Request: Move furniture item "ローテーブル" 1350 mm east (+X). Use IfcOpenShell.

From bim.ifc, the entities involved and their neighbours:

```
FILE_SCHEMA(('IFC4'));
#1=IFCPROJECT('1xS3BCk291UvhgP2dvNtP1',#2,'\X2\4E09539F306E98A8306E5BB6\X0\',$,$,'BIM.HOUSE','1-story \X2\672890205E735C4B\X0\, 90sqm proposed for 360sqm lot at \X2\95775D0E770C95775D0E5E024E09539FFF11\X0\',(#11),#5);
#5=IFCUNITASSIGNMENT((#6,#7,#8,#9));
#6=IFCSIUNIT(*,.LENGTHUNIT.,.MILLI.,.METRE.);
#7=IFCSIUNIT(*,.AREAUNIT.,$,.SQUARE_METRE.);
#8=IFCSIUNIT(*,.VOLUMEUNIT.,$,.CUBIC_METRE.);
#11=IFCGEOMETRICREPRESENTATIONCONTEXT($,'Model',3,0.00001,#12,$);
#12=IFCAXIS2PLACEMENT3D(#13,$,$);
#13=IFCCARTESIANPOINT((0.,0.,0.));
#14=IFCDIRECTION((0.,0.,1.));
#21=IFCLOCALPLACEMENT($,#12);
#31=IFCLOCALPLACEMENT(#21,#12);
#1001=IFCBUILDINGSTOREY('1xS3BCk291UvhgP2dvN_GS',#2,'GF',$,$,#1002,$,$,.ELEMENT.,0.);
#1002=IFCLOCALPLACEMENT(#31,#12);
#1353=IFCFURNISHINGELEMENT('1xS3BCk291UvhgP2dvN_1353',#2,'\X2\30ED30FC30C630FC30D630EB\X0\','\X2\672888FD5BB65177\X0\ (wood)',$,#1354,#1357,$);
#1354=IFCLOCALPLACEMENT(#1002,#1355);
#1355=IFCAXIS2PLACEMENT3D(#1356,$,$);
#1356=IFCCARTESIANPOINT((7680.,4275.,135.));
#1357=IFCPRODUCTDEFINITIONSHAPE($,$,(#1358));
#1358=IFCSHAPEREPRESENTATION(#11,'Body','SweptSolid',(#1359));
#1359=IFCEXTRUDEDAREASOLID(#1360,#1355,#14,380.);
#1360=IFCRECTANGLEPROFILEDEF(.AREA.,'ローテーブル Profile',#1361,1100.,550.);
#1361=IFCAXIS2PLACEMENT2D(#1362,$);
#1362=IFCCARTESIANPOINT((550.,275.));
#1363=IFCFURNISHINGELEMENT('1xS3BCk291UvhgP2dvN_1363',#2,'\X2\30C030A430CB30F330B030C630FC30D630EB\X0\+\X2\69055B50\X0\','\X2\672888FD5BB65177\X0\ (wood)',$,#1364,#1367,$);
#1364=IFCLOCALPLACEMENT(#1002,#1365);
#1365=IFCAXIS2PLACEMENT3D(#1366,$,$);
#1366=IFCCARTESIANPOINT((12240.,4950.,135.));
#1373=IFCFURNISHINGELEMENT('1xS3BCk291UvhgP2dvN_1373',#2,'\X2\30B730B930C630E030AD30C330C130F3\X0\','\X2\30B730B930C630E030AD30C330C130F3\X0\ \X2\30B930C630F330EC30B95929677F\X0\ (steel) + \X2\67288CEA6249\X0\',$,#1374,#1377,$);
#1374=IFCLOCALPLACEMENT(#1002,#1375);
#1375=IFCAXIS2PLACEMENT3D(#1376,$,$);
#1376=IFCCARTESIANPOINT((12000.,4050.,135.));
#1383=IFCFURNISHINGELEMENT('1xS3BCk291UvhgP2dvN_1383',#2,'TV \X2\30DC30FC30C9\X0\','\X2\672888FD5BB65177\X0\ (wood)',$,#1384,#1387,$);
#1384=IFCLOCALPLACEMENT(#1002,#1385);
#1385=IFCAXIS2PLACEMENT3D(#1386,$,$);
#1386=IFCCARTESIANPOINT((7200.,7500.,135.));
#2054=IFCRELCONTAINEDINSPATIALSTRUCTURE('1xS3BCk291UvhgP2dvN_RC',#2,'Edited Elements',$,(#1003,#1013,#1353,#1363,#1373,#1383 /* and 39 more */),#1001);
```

```python
import ifcopenshell
import ifcopenshell.api.geometry
import ifcopenshell.util.placement

model = ifcopenshell.open("bim.ifc")

item = model.by_guid("1xS3BCk291UvhgP2dvN_1353")
matrix = ifcopenshell.util.placement.get_local_placement(item.ObjectPlacement)
matrix[0, 3] += 1350.0
ifcopenshell.api.geometry.edit_object_placement(model, product=item, matrix=matrix, is_si=False)

print(ifcopenshell.util.placement.get_local_placement(item.ObjectPlacement).round(3) + 0.0)

model.write("bim_rev.ifc")
```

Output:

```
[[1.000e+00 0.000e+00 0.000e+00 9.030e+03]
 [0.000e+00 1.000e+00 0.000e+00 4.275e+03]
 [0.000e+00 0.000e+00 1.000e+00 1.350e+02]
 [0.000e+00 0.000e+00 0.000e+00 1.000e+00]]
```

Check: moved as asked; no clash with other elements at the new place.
